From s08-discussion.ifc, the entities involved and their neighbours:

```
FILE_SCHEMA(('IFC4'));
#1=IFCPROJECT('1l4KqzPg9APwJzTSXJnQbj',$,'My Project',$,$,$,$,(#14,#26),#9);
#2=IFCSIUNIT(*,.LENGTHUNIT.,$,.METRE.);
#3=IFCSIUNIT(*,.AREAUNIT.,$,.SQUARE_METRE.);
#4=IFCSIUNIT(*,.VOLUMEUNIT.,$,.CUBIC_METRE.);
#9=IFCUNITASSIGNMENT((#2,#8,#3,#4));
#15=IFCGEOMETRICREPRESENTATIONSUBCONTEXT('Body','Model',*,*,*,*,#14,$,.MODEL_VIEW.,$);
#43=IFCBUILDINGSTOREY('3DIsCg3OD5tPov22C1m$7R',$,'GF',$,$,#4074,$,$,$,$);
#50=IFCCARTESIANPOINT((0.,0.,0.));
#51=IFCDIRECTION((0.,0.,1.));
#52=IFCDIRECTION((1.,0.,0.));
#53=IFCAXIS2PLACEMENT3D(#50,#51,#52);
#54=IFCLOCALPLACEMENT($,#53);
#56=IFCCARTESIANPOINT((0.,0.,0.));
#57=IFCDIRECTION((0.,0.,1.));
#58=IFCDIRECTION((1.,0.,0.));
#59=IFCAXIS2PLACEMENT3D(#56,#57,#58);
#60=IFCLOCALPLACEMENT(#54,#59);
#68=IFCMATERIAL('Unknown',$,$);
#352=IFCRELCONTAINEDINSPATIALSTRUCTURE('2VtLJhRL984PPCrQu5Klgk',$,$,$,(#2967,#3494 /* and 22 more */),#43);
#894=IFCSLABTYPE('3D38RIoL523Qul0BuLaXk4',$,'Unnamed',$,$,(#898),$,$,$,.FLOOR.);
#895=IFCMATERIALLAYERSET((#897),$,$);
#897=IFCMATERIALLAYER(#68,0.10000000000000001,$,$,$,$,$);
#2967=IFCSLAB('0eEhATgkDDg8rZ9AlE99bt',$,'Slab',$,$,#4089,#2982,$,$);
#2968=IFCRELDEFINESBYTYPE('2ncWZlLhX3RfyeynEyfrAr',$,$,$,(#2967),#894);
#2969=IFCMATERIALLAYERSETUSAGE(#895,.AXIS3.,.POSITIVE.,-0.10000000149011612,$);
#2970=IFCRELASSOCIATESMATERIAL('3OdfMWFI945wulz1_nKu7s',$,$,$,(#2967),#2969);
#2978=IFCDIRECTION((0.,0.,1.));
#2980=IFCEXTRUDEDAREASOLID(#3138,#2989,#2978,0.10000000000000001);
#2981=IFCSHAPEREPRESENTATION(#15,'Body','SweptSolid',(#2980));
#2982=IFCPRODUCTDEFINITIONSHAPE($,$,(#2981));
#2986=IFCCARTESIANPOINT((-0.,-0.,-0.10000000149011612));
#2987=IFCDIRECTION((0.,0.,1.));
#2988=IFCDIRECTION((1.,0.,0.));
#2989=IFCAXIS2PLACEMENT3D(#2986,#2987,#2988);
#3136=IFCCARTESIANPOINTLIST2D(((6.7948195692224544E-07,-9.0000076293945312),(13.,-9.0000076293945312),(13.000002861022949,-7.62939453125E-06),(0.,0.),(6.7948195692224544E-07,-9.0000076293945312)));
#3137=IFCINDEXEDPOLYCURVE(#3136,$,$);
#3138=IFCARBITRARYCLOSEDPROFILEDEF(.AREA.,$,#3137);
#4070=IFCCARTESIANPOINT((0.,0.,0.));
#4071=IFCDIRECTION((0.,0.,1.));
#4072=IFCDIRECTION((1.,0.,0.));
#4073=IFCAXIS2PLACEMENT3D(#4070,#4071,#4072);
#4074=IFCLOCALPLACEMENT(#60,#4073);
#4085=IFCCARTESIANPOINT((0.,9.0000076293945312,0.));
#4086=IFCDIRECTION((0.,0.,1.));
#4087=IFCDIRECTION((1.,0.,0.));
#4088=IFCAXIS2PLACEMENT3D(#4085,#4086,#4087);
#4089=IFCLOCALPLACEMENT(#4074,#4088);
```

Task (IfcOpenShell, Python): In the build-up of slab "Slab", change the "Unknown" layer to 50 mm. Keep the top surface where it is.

```python
import ifcopenshell
import ifcopenshell.util.element
import ifcopenshell.util.representation
import ifcopenshell.util.unit

model = ifcopenshell.open("s08-discussion.ifc")
unit_scale = ifcopenshell.util.unit.calculate_unit_scale(model)

layer_set = model.by_id(895)
layer = next(l for l in layer_set.MaterialLayers if l.Material and l.Material.Name == "Unknown")
change = 0.05 / unit_scale - layer.LayerThickness
layer.LayerThickness += change

# Geometry does not follow the layer set by itself.
slabs = [e for e in ifcopenshell.util.element.get_elements_by_material(model, layer_set) if e.is_a("IfcSlab")]
for slab in sorted(slabs, key=lambda e: e.id()):
    body = ifcopenshell.util.representation.get_representation(slab, "Model", "Body")
    solid = body.Items[0]
    old_depth = solid.Depth
    solid.Depth += change
    # Extruded upwards: lower the start of the extrusion so the top stays.
    x, y, z = solid.Position.Location.Coordinates
    solid.Position.Location = model.createIfcCartesianPoint((x, y, z - change))
    print(slab.id(), f"{old_depth:g} -> {solid.Depth:g}")

# The layers are counted up from the underside, which has moved.
for usage in {ifcopenshell.util.element.get_material(slab) for slab in slabs}:
    usage.OffsetFromReferenceLine -= change

model.write("s08-discussion_rev.ifc")
```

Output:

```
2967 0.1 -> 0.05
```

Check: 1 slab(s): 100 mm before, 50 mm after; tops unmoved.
